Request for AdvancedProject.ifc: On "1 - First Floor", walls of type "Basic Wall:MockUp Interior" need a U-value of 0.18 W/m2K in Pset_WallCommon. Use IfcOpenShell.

First a look at what the model holds.

```python
import ifcopenshell
import ifcopenshell.util.element

model = ifcopenshell.open("AdvancedProject.ifc")
print(model.schema)
storey = next(s for s in model.by_type("IfcBuildingStorey") if s.Name == "1 - First Floor")
walls = [e for e in ifcopenshell.util.element.get_decomposition(storey) if e.is_a("IfcWall")]
seen = {}
for e in walls:
    element_type = ifcopenshell.util.element.get_type(e)
    key = (element_type.Name if element_type != e and element_type else None, ifcopenshell.util.element.get_pset(e, "Pset_WallCommon", "ThermalTransmittance"))
    seen[key] = seen.get(key, 0) + 1
for (name, value), count in sorted(seen.items(), key=str):
    print(count, "x", name, "|", value)
```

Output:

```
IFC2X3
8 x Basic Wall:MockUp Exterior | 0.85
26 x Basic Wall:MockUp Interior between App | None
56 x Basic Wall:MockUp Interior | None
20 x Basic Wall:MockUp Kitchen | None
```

```python
import ifcopenshell
import ifcopenshell.api.pset
import ifcopenshell.util.element

model = ifcopenshell.open("AdvancedProject.ifc")

storey = next(s for s in model.by_type("IfcBuildingStorey") if s.Name == "1 - First Floor")
walls = [e for e in ifcopenshell.util.element.get_decomposition(storey) if e.is_a("IfcWall")]

count = 0
for e in walls:
    element_type = ifcopenshell.util.element.get_type(e)
    if element_type in (None, e) or element_type.Name != "Basic Wall:MockUp Interior":
        continue
    # add_pset returns the element's existing set when there is one.
    pset = ifcopenshell.api.pset.add_pset(model, product=e, name="Pset_WallCommon")
    ifcopenshell.api.pset.edit_pset(model, pset=pset, properties={"ThermalTransmittance": 0.18})
    count += 1

print(count, "walls updated")

model.write("AdvancedProject_updated.ifc")
```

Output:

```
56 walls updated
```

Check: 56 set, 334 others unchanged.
